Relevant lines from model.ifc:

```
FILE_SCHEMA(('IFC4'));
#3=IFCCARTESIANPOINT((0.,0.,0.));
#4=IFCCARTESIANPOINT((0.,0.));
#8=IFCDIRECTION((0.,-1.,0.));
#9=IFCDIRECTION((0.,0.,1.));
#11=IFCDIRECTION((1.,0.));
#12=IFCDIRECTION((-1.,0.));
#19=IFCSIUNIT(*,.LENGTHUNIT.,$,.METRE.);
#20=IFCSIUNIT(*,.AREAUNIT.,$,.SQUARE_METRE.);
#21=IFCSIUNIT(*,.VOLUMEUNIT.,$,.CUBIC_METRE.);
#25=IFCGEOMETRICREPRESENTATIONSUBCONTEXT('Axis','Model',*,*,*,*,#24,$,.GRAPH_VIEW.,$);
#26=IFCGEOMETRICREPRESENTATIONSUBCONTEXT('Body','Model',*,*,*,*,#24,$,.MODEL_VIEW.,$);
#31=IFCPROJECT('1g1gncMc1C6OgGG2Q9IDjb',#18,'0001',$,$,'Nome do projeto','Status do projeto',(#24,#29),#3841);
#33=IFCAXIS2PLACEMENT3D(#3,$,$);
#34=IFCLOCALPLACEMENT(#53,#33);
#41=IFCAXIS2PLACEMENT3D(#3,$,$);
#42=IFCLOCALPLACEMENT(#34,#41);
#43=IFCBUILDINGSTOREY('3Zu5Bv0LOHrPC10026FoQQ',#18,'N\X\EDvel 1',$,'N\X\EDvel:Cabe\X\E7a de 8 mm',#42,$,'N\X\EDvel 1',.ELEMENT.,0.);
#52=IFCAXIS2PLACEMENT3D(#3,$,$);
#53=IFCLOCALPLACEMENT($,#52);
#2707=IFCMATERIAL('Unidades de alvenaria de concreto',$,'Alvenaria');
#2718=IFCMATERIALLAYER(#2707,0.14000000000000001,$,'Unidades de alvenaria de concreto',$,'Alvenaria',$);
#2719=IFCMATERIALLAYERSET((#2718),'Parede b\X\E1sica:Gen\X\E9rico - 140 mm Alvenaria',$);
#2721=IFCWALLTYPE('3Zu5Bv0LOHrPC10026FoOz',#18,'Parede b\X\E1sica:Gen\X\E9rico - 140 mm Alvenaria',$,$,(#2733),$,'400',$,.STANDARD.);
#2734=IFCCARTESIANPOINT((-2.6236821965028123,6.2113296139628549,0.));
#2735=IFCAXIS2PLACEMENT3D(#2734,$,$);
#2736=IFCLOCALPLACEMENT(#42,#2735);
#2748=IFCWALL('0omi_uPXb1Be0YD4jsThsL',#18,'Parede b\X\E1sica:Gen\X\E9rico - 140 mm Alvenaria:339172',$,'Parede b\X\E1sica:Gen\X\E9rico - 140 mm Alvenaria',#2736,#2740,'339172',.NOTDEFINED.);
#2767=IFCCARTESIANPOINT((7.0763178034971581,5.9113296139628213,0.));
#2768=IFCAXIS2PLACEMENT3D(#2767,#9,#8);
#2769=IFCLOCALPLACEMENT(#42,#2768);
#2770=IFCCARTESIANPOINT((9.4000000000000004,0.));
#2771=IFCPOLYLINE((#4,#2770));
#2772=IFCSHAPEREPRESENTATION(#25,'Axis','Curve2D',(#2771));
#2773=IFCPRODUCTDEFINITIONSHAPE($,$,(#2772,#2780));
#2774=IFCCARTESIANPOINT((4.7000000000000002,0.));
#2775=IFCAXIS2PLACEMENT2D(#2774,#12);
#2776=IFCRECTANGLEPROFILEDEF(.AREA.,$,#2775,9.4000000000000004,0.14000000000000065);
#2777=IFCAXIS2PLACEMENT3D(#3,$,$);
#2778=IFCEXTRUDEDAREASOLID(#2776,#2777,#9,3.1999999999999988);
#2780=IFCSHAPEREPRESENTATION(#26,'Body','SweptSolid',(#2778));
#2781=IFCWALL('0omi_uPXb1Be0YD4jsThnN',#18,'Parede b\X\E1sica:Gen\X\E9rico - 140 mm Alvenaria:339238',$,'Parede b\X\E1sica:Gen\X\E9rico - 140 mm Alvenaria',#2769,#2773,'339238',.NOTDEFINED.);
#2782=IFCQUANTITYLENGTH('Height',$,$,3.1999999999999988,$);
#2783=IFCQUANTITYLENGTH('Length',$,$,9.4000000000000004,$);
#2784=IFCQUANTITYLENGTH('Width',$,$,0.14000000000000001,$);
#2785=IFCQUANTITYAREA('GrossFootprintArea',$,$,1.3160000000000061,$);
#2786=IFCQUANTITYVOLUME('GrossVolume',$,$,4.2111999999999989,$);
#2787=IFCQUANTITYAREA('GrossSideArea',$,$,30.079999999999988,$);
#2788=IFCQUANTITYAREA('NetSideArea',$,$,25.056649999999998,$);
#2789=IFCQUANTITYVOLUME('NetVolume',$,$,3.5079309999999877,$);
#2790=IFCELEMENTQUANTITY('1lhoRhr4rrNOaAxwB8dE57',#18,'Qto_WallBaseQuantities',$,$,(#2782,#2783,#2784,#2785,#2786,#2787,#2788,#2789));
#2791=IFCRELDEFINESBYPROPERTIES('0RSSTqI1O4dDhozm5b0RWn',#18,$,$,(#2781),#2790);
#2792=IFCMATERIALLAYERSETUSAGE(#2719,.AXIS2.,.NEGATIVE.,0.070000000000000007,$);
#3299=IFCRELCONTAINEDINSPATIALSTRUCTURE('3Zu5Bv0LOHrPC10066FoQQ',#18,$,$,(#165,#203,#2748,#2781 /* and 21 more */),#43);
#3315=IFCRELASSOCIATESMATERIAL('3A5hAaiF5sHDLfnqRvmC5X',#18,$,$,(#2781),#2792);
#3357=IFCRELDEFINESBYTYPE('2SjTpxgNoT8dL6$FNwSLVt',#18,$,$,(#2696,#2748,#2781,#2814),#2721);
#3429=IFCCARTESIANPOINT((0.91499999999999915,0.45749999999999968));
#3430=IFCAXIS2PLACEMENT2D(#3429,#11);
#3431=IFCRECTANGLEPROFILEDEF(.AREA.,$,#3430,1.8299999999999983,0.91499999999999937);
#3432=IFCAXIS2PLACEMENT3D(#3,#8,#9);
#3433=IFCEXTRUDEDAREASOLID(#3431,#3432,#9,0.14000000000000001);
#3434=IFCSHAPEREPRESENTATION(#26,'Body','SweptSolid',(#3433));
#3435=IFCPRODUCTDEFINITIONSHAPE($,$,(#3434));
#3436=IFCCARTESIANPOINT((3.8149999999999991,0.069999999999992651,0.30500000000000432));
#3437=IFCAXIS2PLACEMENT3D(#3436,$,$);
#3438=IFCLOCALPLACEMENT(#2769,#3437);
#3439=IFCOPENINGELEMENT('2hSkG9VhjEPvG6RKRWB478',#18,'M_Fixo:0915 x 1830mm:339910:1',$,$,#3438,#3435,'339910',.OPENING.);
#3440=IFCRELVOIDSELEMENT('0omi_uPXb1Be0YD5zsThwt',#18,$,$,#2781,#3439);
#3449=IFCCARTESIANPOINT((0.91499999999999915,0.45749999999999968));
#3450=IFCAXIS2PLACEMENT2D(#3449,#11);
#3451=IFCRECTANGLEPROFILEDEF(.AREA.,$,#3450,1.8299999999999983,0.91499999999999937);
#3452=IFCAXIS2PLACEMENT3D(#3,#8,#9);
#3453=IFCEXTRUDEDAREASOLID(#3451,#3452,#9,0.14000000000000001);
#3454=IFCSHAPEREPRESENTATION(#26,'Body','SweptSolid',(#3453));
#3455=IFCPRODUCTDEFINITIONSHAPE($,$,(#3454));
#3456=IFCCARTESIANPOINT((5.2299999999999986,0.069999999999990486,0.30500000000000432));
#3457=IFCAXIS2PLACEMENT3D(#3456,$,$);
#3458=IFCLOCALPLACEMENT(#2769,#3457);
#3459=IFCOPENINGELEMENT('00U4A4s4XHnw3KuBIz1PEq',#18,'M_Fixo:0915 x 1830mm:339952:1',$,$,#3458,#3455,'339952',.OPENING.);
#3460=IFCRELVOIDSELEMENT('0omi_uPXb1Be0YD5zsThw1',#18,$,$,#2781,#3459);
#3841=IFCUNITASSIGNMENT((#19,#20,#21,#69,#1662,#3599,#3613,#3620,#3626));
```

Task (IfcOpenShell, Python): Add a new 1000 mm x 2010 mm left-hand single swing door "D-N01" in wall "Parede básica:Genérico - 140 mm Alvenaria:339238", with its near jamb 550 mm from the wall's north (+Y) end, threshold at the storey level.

```python
import numpy as np
import ifcopenshell
import ifcopenshell.api.feature
import ifcopenshell.api.geometry
import ifcopenshell.api.pset
import ifcopenshell.api.root
import ifcopenshell.api.spatial
import ifcopenshell.geom
import ifcopenshell.util.element
import ifcopenshell.util.placement
import ifcopenshell.util.representation
import ifcopenshell.util.shape
import ifcopenshell.util.unit

model = ifcopenshell.open("model.ifc")
unit_scale = ifcopenshell.util.unit.calculate_unit_scale(model)
area_scale = ifcopenshell.util.unit.calculate_unit_scale(model, "AREAUNIT")
volume_scale = ifcopenshell.util.unit.calculate_unit_scale(model, "VOLUMEUNIT")
settings = ifcopenshell.geom.settings()


def volume(element):
    """Net volume in cubic metres, openings subtracted."""
    shape = ifcopenshell.geom.create_shape(settings, element)
    return ifcopenshell.util.shape.get_volume(shape.geometry)


wall = model.by_guid("0omi_uPXb1Be0YD4jsThnN")
storey = ifcopenshell.util.element.get_container(wall, ifc_class="IfcBuildingStorey")
context = ifcopenshell.util.representation.get_context(model, "Model", "Body", "MODEL_VIEW")
before = volume(wall)

width, height, from_end, sill = 1, 2.01, 0.55, 0.0  # metres

# The wall runs along its own X axis, and the end named is its -X end.
wall_shape = ifcopenshell.geom.create_shape(settings, wall)
x, y, z = ifcopenshell.util.shape.get_vertices(wall_shape.geometry).T
start = x.min() + from_end
face, thickness = float(y.min()), float(y.max() - y.min())
wall_matrix = ifcopenshell.util.placement.get_local_placement(wall.ObjectPlacement)
level = ifcopenshell.util.placement.get_local_placement(storey.ObjectPlacement)[2, 3]


def in_wall(x, y):
    """Placement at x, y metres in the wall's axes, at sill height."""
    matrix = wall_matrix.copy()
    matrix[:, 3] = wall_matrix @ np.array([x / unit_scale, y / unit_scale, 0.0, 1.0])
    matrix[2, 3] = level + sill / unit_scale
    return matrix


# Opening: a box that overshoots both wall faces by 50 mm.
opening = ifcopenshell.api.root.create_entity(model, ifc_class="IfcOpeningElement", predefined_type="OPENING")
box = ifcopenshell.api.geometry.add_wall_representation(
    model, context=context, length=width, height=height, thickness=thickness + 0.1
)
ifcopenshell.api.geometry.assign_representation(model, product=opening, representation=box)
ifcopenshell.api.geometry.edit_object_placement(model, product=opening, matrix=in_wall(start, face - 0.05), is_si=False)
ifcopenshell.api.feature.add_feature(model, feature=opening, element=wall)

door = ifcopenshell.api.root.create_entity(model, ifc_class="IfcDoor", name="D-N01", predefined_type="DOOR")
door.OverallWidth, door.OverallHeight = width / unit_scale, height / unit_scale
door.OperationType = "SINGLE_SWING_LEFT"
body = ifcopenshell.api.geometry.add_door_representation(
    model,
    context=context,
    overall_width=door.OverallWidth,
    overall_height=door.OverallHeight,
    operation_type="SINGLE_SWING_LEFT",
    lining_properties={"LiningDepth": thickness / unit_scale, "ThresholdDepth": thickness / unit_scale},
)
ifcopenshell.api.geometry.assign_representation(model, product=door, representation=body)
ifcopenshell.api.spatial.assign_container(model, products=[door], relating_structure=storey)
ifcopenshell.api.feature.add_filling(model, opening=opening, element=door)

# The lining spans the wall, so the door starts at the wall face.
ifcopenshell.api.geometry.edit_object_placement(model, product=door, matrix=in_wall(start, face), is_si=False)

after = volume(wall)

# Update the wall's stored quantities.
qto = model.by_id(ifcopenshell.util.element.get_pset(wall, "Qto_WallBaseQuantities", should_inherit=False)["id"])
ifcopenshell.api.pset.edit_qto(model, qto=qto, properties={
    "NetSideArea": after / thickness / area_scale,
    "NetVolume": after / volume_scale,
})

print(f"wall volume {before:.3f} -> {after:.3f} m3")

model.write("model_rev.ifc")
```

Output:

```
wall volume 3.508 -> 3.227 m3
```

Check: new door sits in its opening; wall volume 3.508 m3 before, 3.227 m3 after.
